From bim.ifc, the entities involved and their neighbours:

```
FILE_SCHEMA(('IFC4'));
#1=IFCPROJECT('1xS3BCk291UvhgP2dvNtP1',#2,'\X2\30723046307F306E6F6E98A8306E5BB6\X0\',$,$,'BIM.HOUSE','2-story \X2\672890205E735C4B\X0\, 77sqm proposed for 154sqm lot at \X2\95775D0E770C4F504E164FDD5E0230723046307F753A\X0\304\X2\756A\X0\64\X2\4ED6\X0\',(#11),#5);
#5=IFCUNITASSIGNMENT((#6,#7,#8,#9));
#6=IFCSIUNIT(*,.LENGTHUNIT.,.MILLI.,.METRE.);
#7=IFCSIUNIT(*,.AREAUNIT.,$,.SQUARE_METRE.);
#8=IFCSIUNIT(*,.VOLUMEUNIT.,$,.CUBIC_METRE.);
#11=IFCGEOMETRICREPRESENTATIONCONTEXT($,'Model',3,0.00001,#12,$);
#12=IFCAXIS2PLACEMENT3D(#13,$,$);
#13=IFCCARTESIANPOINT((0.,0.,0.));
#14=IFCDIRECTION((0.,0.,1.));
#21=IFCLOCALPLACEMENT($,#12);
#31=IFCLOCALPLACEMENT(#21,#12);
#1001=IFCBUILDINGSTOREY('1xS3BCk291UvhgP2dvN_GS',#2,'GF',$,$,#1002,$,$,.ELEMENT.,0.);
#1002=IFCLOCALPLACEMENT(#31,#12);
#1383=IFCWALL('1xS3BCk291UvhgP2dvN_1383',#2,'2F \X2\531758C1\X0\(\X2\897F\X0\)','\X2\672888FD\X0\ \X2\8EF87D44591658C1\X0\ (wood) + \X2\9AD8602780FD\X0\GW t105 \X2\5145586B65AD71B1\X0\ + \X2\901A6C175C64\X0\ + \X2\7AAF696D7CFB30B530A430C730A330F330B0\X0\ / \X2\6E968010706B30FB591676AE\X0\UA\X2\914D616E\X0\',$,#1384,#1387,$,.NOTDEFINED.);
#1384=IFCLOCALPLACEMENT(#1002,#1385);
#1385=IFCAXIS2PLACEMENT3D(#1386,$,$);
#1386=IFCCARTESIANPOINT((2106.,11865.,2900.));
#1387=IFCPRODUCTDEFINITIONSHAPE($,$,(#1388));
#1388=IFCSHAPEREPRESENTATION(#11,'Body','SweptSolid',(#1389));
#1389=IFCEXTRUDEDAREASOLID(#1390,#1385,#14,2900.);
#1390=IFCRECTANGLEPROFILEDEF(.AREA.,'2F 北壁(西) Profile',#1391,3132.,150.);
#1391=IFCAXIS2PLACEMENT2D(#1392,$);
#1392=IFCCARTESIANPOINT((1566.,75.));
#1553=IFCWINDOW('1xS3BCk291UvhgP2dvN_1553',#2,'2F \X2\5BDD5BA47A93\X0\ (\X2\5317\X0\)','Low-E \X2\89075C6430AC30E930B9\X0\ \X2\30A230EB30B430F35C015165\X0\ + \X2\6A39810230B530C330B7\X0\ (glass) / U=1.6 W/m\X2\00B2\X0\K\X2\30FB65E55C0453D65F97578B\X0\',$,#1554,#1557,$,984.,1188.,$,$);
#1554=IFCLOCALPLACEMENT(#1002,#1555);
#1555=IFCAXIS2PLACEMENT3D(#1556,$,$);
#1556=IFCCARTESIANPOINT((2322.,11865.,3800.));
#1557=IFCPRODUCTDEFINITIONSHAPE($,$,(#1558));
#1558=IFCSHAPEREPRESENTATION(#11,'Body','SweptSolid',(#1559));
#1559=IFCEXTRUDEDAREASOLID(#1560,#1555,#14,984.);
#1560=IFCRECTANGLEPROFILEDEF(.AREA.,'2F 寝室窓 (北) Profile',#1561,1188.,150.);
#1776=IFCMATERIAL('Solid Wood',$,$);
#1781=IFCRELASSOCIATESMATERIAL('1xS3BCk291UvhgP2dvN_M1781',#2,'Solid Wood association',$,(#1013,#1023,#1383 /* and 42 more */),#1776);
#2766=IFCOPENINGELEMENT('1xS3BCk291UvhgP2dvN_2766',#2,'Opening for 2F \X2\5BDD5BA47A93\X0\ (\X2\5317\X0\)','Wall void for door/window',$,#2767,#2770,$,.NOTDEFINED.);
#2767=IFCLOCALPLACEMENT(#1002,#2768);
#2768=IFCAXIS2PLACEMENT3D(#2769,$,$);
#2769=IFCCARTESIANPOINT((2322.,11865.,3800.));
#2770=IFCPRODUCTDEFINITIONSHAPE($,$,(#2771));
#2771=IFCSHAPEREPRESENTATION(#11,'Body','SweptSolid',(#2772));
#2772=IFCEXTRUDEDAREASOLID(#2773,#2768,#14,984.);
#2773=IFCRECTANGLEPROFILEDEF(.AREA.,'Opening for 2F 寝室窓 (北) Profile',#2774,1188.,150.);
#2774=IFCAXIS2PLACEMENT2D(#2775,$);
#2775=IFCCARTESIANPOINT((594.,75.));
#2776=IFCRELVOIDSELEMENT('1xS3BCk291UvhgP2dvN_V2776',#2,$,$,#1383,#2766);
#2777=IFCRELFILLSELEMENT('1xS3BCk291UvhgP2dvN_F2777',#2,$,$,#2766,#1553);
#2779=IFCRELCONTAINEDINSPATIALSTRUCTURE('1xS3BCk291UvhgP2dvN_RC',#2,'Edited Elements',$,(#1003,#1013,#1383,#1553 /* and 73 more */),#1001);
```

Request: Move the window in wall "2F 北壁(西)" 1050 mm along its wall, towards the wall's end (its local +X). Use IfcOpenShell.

```python
import ifcopenshell
import ifcopenshell.api.geometry
import ifcopenshell.util.placement
import ifcopenshell.util.unit

model = ifcopenshell.open("bim.ifc")
unit_scale = ifcopenshell.util.unit.calculate_unit_scale(model)

window = model.by_guid("1xS3BCk291UvhgP2dvN_1553")
opening = window.FillsVoids[0].RelatingOpeningElement
wall = opening.VoidsElements[0].RelatingBuildingElement

wall_matrix = ifcopenshell.util.placement.get_local_placement(wall.ObjectPlacement)
shift = wall_matrix[:3, 0] * 1.05 / unit_scale
before = ifcopenshell.util.placement.get_local_placement(window.ObjectPlacement)[:3, 3].copy()

# The window is not placed relative to its opening, so move both.
for product in (opening, window):
    matrix = ifcopenshell.util.placement.get_local_placement(product.ObjectPlacement)
    matrix[:3, 3] += shift
    ifcopenshell.api.geometry.edit_object_placement(model, product=product, matrix=matrix, is_si=False)

after = ifcopenshell.util.placement.get_local_placement(window.ObjectPlacement)[:3, 3]
print("window moved by", (after - before).round(3) + 0.0)

model.write("bim_edited.ifc")
```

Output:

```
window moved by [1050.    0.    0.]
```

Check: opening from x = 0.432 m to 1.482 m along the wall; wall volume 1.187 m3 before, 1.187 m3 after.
